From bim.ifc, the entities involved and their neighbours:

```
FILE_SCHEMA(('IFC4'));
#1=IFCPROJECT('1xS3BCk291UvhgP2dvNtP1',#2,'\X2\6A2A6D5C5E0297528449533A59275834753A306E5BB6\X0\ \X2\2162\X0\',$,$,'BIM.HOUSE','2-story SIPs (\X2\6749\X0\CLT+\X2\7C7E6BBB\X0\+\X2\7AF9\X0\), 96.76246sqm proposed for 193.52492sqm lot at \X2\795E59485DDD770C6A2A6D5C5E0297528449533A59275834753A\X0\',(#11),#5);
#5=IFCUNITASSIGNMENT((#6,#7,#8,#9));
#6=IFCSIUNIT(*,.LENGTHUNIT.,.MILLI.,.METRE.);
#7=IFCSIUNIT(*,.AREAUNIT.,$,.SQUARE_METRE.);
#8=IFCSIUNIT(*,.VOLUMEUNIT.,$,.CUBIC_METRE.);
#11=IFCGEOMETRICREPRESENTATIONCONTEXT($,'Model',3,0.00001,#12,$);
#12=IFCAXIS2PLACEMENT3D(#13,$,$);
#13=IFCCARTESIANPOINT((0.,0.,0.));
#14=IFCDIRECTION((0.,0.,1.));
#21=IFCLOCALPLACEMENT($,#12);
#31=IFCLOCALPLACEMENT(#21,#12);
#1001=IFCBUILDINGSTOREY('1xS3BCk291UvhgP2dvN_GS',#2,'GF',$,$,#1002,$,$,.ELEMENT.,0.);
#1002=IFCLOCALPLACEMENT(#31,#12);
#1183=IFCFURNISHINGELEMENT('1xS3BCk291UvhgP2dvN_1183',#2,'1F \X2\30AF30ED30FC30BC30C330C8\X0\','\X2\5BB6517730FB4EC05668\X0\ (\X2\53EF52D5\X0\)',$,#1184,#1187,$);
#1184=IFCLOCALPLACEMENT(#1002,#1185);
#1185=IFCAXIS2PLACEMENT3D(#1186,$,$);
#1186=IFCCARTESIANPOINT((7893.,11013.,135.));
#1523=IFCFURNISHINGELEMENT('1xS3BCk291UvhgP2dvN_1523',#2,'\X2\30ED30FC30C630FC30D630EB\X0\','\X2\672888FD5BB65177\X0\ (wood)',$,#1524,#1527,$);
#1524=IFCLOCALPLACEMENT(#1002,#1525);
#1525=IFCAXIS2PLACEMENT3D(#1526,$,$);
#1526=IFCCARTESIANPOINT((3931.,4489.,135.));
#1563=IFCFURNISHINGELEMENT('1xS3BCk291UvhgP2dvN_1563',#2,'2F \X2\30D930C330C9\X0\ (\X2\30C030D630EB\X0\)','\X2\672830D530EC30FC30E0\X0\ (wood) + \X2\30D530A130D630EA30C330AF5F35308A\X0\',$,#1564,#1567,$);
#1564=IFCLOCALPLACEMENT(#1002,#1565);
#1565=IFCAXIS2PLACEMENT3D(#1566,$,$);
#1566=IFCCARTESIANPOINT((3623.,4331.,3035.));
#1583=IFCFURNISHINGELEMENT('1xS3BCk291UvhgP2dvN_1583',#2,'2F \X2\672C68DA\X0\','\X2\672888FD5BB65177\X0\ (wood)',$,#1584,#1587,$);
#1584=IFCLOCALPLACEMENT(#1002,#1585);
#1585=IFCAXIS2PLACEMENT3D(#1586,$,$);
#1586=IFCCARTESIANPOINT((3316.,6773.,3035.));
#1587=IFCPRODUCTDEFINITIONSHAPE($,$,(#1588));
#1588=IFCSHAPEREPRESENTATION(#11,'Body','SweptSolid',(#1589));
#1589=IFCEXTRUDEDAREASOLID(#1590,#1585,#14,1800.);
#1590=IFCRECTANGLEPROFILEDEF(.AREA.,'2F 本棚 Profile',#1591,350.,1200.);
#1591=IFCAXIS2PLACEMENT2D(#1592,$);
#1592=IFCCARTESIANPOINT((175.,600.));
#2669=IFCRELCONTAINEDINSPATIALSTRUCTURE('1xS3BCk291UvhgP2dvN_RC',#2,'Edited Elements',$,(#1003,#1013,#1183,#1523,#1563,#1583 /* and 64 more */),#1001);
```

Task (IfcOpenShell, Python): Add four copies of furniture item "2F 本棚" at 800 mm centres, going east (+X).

```python
import numpy as np
import ifcopenshell
import ifcopenshell.api.geometry
import ifcopenshell.api.root
import ifcopenshell.util.element
import ifcopenshell.util.placement
import ifcopenshell.util.unit

model = ifcopenshell.open("bim.ifc")
unit_scale = ifcopenshell.util.unit.calculate_unit_scale(model)


def reuse_history(source, copy):
    """copy_class also copies each property set's owner history, people and application; keep the originals."""
    for rel in copy.IsDefinedBy:
        if rel.is_a("IfcRelDefinesByProperties") and (history := rel.RelatingPropertyDefinition.OwnerHistory):
            rel.RelatingPropertyDefinition.OwnerHistory = source.OwnerHistory
            ifcopenshell.util.element.remove_deep2(model, history)


source = model.by_id(1583)
base = ifcopenshell.util.placement.get_local_placement(source.ObjectPlacement)
step = np.array([1.0, 0.0, 0.0]) * 0.8 / unit_scale

for i in range(1, 5):
    copy = ifcopenshell.api.root.copy_class(model, product=source)
    copy.Representation = ifcopenshell.util.element.copy_deep(
        model, source.Representation, exclude=["IfcGeometricRepresentationContext", "IfcRepresentationMap"]
    )
    reuse_history(source, copy)
    matrix = base.copy()
    matrix[:3, 3] += i * step
    print("added at", matrix[:3, 3].round(3) + 0.0)
    ifcopenshell.api.geometry.edit_object_placement(model, product=copy, matrix=matrix, is_si=False)

model.write("bim_v2.ifc")
```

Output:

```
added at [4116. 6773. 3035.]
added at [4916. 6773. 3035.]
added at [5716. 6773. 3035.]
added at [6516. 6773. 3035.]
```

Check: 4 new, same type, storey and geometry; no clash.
